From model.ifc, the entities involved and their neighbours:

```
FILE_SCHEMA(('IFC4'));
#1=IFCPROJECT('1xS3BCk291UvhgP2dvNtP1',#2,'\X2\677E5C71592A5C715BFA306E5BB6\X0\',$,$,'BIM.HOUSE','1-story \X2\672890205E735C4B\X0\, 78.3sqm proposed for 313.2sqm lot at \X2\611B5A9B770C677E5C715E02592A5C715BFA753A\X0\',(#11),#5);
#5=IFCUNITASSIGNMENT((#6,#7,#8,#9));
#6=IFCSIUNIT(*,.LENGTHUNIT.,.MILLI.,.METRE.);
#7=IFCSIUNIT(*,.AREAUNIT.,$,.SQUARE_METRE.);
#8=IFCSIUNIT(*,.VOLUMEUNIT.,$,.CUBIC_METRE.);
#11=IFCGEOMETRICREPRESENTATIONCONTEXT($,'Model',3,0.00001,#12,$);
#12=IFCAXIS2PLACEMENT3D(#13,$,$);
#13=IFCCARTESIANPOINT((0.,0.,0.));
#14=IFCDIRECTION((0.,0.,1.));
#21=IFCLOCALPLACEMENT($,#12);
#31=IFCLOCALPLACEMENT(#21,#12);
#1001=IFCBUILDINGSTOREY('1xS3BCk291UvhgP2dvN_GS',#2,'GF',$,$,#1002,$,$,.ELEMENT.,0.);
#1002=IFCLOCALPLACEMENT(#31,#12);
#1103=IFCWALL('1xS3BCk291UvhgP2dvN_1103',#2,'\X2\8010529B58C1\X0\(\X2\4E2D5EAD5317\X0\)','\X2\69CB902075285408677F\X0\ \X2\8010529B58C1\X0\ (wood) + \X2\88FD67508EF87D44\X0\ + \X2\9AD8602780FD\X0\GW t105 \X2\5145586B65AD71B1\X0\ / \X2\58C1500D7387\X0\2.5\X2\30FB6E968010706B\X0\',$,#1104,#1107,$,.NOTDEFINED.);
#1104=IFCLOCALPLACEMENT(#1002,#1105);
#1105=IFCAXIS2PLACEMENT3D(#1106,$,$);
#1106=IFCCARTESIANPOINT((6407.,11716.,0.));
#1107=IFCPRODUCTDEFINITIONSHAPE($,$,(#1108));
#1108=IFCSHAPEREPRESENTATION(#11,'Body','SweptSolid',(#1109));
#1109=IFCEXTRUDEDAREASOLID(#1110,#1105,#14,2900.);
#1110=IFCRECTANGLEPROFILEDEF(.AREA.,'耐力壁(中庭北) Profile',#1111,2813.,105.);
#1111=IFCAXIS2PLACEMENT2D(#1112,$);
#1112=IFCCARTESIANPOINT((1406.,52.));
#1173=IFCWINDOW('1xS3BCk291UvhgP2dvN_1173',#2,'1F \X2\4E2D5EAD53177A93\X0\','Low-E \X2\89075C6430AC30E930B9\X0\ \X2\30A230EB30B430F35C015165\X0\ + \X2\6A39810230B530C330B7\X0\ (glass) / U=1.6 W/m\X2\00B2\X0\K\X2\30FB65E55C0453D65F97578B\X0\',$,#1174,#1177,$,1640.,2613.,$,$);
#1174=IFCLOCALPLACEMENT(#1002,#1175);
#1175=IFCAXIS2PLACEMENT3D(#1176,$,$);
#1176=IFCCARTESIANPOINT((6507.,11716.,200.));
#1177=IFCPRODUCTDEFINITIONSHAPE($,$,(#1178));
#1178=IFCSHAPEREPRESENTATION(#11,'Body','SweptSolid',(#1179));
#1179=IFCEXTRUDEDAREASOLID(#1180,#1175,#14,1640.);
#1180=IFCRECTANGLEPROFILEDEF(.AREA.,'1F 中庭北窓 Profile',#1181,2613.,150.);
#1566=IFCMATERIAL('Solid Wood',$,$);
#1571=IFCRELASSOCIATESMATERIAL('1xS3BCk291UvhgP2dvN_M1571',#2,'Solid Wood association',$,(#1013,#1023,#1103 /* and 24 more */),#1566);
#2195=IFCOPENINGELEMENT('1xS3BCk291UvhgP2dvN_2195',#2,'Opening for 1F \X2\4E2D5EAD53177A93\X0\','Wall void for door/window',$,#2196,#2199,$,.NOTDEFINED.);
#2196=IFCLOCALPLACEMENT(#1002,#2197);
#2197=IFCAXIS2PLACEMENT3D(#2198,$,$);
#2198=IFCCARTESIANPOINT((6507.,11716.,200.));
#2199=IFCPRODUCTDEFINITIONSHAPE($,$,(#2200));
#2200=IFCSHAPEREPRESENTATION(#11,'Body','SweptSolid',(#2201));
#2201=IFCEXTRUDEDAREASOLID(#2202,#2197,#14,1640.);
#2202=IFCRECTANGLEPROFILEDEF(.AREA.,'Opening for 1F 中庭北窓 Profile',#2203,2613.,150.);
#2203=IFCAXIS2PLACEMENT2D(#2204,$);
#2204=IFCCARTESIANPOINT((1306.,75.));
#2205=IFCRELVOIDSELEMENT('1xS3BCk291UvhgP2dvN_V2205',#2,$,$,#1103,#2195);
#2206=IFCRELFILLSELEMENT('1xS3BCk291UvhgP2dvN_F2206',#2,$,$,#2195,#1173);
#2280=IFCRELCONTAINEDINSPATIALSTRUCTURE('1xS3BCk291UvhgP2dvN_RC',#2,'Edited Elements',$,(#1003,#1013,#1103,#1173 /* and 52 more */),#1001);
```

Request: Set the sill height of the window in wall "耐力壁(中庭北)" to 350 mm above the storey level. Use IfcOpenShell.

```python
import numpy as np
import ifcopenshell
import ifcopenshell.api.geometry
import ifcopenshell.geom
import ifcopenshell.util.element
import ifcopenshell.util.placement
import ifcopenshell.util.shape
import ifcopenshell.util.unit

model = ifcopenshell.open("model.ifc")
unit_scale = ifcopenshell.util.unit.calculate_unit_scale(model)

window = model.by_guid("1xS3BCk291UvhgP2dvN_1173")
opening = window.FillsVoids[0].RelatingOpeningElement
storey = ifcopenshell.util.element.get_container(window, ifc_class="IfcBuildingStorey")
level = ifcopenshell.util.placement.get_local_placement(storey.ObjectPlacement)[2, 3]

# The opening's origin need not be at the sill, so measure its lowest point.
shape = ifcopenshell.geom.create_shape(ifcopenshell.geom.settings(), opening)
bottom = ifcopenshell.util.shape.get_shape_bottom_elevation(shape, shape.geometry) / unit_scale
dz = level + 0.35 / unit_scale - bottom

shift = np.array([0.0, 0.0, dz])
# The window is not placed relative to its opening, so move both.
for product in (opening, window):
    matrix = ifcopenshell.util.placement.get_local_placement(product.ObjectPlacement)
    matrix[:3, 3] += shift
    ifcopenshell.api.geometry.edit_object_placement(model, product=product, matrix=matrix, is_si=False)

print(f"moved by {dz * unit_scale:+.3f} m")

model.write("model_rev.ifc")
```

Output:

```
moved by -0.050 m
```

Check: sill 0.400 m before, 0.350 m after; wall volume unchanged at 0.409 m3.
